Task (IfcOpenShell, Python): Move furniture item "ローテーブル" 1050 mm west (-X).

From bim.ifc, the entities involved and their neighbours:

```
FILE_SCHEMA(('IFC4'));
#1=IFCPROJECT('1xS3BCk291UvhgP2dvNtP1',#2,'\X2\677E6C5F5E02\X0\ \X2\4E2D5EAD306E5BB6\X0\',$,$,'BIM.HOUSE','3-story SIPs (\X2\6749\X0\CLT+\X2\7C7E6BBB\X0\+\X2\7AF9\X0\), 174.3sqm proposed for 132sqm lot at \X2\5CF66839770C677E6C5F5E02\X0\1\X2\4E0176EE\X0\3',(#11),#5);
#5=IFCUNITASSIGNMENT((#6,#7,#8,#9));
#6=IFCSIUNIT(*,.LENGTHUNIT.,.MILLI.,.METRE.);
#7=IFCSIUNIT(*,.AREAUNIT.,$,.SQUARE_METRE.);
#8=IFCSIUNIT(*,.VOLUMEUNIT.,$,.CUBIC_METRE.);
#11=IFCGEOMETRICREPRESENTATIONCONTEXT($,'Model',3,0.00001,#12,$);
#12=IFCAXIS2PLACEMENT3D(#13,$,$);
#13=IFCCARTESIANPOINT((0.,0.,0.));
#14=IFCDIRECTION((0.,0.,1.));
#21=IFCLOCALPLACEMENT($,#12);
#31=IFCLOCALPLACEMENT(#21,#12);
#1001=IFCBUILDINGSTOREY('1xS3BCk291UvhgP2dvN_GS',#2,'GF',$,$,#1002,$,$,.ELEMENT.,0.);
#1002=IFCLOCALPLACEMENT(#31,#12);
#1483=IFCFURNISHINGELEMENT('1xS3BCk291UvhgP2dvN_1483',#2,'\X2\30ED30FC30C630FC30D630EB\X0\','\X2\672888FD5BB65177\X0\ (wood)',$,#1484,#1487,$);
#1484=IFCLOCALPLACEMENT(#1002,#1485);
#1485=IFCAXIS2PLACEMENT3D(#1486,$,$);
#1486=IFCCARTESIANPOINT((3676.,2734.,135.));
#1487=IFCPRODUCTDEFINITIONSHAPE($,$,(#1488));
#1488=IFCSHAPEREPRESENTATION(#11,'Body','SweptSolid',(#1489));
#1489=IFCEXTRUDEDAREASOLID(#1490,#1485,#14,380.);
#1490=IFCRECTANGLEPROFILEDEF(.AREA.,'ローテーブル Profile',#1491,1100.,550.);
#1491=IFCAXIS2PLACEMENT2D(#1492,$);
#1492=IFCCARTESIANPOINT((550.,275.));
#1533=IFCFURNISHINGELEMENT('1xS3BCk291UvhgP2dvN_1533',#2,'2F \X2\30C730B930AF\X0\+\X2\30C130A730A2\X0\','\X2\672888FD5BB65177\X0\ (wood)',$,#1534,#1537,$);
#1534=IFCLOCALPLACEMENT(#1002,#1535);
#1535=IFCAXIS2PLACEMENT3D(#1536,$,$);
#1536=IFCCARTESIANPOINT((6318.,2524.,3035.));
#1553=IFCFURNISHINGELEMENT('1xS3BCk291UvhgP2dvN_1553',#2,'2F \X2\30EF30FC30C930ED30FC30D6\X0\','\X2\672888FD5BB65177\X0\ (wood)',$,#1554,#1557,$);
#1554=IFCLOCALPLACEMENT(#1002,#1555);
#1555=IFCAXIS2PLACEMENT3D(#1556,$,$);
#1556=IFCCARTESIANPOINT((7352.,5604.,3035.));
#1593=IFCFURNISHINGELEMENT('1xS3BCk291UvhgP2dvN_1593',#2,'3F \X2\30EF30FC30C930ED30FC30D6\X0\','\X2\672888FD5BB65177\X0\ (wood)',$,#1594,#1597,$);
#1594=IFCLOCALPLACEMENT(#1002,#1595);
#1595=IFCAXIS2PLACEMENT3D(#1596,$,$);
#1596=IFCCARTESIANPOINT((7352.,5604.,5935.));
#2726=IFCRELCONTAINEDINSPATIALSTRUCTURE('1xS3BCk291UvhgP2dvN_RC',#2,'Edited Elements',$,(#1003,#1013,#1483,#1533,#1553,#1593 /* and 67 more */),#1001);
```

```python
import ifcopenshell
import ifcopenshell.api.geometry
import ifcopenshell.util.placement
import ifcopenshell.util.unit

model = ifcopenshell.open("bim.ifc")
unit_scale = ifcopenshell.util.unit.calculate_unit_scale(model)

item = model.by_guid("1xS3BCk291UvhgP2dvN_1483")
matrix = ifcopenshell.util.placement.get_local_placement(item.ObjectPlacement)
matrix[0, 3] -= 1.05 / unit_scale
ifcopenshell.api.geometry.edit_object_placement(model, product=item, matrix=matrix, is_si=False)

print(ifcopenshell.util.placement.get_local_placement(item.ObjectPlacement).round(3) + 0.0)

model.write("bim_rev.ifc")
```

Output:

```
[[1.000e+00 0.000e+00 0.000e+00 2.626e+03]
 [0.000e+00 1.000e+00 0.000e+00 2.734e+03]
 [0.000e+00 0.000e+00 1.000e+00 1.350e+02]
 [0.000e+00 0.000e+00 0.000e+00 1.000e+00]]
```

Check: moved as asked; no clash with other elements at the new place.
